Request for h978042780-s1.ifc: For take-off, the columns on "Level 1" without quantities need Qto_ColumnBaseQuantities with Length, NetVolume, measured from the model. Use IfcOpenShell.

First a look at what the model holds.

```python
import ifcopenshell
import ifcopenshell.util.element
import ifcopenshell.util.unit

model = ifcopenshell.open("h978042780-s1.ifc")
print(model.schema)
for unit_type in ("LENGTHUNIT", "AREAUNIT", "VOLUMEUNIT"):
    print(unit_type, ifcopenshell.util.unit.calculate_unit_scale(model, unit_type))
storey = next(s for s in model.by_type("IfcBuildingStorey") if s.Name == "Level 1")
columns = [e for e in ifcopenshell.util.element.get_decomposition(storey) if e.is_a("IfcColumn")]
for e in sorted(columns, key=lambda e: e.id()):
    print(e.id(), e.is_a(), e.Name, list(ifcopenshell.util.element.get_psets(e, qtos_only=True)), sep=" | ")
```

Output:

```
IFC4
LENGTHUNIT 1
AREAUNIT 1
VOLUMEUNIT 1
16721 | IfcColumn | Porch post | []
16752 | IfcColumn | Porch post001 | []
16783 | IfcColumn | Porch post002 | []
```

```python
import ifcopenshell
import ifcopenshell.api.pset
import ifcopenshell.geom
import ifcopenshell.util.element
import ifcopenshell.util.shape
import ifcopenshell.util.unit

model = ifcopenshell.open("h978042780-s1.ifc")
unit_scale = ifcopenshell.util.unit.calculate_unit_scale(model)
volume_scale = ifcopenshell.util.unit.calculate_unit_scale(model, "VOLUMEUNIT")
settings = ifcopenshell.geom.settings()

storey = next(s for s in model.by_type("IfcBuildingStorey") if s.Name == "Level 1")
columns = [e for e in ifcopenshell.util.element.get_decomposition(storey) if e.is_a("IfcColumn")]

for e in sorted(columns, key=lambda e: e.id()):
    if ifcopenshell.util.element.get_psets(e, qtos_only=True, should_inherit=False):
        continue
    # Geometry comes back in metres, in the element's own axes.
    shape = ifcopenshell.geom.create_shape(settings, e)
    values = {
        "Length": ifcopenshell.util.shape.get_z(shape.geometry) / unit_scale,
        "NetVolume": ifcopenshell.util.shape.get_volume(shape.geometry) / volume_scale,
    }
    qto = ifcopenshell.api.pset.add_qto(model, product=e, name="Qto_ColumnBaseQuantities")
    ifcopenshell.api.pset.edit_qto(model, qto=qto, properties=values)
    print(e.id(), {k: round(v, 3) for k, v in values.items()})

model.write("h978042780-s1_v2.ifc")
```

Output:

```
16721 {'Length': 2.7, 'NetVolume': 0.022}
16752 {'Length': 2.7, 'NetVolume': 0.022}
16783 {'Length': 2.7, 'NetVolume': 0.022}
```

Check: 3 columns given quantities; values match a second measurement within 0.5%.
